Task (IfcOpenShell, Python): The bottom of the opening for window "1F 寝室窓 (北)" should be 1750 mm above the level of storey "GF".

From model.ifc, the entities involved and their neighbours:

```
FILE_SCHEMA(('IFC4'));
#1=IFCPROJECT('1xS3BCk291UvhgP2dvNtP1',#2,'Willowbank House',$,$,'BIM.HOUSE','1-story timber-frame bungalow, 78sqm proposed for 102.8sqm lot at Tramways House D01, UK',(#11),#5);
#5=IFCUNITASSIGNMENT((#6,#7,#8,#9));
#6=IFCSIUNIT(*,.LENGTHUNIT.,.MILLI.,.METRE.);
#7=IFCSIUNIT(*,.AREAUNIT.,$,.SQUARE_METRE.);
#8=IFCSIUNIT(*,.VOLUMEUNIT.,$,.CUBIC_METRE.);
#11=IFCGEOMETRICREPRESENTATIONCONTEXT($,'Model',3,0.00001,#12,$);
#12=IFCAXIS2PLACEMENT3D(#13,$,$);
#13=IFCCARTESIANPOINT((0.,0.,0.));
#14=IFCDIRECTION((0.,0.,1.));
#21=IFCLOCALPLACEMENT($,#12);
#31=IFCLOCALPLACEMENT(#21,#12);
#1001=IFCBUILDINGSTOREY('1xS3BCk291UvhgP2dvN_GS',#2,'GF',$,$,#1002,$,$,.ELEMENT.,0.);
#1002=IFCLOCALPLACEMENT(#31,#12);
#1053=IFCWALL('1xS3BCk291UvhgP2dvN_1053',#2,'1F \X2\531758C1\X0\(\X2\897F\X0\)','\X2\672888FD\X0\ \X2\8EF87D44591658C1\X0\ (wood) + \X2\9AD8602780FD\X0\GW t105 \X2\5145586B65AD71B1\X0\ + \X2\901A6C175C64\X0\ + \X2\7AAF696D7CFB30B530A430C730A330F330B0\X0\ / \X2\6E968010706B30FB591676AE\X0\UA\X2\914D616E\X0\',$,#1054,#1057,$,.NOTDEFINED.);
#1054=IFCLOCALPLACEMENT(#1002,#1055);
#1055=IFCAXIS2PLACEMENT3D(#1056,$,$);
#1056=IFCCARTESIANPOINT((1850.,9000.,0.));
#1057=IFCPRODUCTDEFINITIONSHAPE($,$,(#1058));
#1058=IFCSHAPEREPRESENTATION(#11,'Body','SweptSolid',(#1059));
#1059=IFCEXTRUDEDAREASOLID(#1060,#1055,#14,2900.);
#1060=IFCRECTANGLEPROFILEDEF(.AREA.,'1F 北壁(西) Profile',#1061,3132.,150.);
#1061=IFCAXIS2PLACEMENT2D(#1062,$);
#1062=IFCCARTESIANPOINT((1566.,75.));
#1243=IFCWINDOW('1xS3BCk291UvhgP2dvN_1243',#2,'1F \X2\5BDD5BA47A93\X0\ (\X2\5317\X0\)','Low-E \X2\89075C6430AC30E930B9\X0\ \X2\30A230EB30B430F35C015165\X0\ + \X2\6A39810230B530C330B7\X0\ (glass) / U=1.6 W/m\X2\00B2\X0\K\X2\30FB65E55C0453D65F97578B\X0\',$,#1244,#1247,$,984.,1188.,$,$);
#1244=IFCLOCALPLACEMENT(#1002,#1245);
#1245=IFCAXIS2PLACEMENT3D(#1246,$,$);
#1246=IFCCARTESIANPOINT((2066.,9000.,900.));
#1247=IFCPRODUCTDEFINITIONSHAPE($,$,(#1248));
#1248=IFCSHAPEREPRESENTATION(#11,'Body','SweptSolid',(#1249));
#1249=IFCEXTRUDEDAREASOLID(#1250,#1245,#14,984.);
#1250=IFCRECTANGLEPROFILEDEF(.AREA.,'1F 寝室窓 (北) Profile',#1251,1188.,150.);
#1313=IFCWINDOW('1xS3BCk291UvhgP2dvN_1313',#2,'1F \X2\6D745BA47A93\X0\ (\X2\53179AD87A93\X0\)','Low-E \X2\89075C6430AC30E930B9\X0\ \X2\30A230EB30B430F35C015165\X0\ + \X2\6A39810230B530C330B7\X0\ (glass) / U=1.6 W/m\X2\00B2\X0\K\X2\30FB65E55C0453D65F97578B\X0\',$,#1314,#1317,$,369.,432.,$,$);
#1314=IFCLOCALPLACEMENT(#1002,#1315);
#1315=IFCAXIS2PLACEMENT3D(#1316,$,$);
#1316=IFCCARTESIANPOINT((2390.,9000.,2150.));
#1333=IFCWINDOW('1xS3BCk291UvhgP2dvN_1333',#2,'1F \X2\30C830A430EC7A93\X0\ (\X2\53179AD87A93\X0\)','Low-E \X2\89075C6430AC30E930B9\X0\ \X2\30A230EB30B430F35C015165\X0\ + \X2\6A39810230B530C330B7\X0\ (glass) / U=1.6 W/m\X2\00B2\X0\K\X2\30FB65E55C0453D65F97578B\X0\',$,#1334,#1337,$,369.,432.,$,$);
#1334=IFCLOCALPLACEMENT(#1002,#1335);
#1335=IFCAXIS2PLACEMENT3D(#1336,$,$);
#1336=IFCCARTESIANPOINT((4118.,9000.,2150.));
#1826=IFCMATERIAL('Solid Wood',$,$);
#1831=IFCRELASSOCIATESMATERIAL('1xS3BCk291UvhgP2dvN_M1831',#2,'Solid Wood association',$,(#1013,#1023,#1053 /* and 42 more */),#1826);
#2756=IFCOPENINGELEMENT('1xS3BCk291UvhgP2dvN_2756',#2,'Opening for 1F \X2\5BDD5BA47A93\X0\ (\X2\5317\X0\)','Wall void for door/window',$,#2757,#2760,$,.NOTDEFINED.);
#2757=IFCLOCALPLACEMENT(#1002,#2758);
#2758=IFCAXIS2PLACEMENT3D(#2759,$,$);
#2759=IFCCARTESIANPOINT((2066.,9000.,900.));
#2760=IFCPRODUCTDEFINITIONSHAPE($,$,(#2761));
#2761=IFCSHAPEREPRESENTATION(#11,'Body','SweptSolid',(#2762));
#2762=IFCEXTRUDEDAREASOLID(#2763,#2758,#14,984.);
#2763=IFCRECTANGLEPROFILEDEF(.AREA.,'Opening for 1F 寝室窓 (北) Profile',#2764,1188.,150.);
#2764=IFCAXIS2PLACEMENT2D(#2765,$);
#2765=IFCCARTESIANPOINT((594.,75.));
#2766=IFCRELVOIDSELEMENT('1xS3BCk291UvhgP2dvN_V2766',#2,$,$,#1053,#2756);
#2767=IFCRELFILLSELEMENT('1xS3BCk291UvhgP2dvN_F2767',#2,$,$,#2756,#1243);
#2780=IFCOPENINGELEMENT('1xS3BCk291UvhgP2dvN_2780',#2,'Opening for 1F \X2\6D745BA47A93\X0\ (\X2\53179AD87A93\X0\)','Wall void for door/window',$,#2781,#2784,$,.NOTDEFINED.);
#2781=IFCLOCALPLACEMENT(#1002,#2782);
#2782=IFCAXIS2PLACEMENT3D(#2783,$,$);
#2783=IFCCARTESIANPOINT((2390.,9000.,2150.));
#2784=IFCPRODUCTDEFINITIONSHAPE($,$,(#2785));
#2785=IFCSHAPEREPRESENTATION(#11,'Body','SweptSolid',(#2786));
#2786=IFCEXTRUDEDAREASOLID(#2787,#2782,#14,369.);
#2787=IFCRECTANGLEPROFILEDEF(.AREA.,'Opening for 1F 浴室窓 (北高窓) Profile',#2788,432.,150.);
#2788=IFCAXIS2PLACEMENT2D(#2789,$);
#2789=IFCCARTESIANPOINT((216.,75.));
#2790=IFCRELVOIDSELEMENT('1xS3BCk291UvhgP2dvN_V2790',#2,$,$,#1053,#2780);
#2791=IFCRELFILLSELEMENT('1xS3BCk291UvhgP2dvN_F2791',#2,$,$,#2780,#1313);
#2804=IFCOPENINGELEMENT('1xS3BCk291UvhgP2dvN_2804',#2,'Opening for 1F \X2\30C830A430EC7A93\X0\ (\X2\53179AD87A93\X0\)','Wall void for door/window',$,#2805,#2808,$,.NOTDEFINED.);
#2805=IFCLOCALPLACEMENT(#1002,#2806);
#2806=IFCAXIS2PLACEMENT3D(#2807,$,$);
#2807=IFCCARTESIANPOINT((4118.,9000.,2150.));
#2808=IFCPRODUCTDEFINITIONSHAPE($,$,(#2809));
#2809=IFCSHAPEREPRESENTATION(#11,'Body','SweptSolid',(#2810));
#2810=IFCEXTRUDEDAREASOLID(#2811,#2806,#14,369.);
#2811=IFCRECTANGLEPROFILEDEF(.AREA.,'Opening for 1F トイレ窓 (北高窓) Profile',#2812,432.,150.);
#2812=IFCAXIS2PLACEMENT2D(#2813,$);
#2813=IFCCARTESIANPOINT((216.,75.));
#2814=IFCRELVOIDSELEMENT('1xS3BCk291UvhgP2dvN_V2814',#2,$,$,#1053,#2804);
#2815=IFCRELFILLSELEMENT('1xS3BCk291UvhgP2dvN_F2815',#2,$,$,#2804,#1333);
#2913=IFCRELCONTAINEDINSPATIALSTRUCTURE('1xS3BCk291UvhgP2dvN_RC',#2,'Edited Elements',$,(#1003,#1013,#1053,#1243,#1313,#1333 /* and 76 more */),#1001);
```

```python
import numpy as np
import ifcopenshell
import ifcopenshell.api.geometry
import ifcopenshell.geom
import ifcopenshell.util.element
import ifcopenshell.util.placement
import ifcopenshell.util.shape
import ifcopenshell.util.unit

model = ifcopenshell.open("model.ifc")
unit_scale = ifcopenshell.util.unit.calculate_unit_scale(model)

window = model.by_guid("1xS3BCk291UvhgP2dvN_1243")
opening = window.FillsVoids[0].RelatingOpeningElement
storey = ifcopenshell.util.element.get_container(window, ifc_class="IfcBuildingStorey")
level = ifcopenshell.util.placement.get_local_placement(storey.ObjectPlacement)[2, 3]

# The opening's origin need not be at the sill, so measure its lowest point.
shape = ifcopenshell.geom.create_shape(ifcopenshell.geom.settings(), opening)
bottom = ifcopenshell.util.shape.get_shape_bottom_elevation(shape, shape.geometry) / unit_scale
dz = level + 1.75 / unit_scale - bottom

shift = np.array([0.0, 0.0, dz])
# The window is not placed relative to its opening, so move both.
for product in (opening, window):
    matrix = ifcopenshell.util.placement.get_local_placement(product.ObjectPlacement)
    matrix[:3, 3] += shift
    ifcopenshell.api.geometry.edit_object_placement(model, product=product, matrix=matrix, is_si=False)

print(f"moved by {dz * unit_scale:+.3f} m")

model.write("model_rev.ifc")
```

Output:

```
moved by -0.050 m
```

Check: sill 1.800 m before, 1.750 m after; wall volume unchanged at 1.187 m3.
